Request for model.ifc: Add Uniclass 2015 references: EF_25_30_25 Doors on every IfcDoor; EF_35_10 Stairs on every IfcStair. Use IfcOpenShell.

First a look at what the model holds.

```python
import ifcopenshell

model = ifcopenshell.open("model.ifc")
print(model.schema)
print("classifications:", [c.Name for c in model.by_type("IfcClassification")])
for ifc_class in ("IfcDoor", "IfcRoof", "IfcStair", "IfcWall", "IfcWindow"):
    print(ifc_class, len(model.by_type(ifc_class)))
```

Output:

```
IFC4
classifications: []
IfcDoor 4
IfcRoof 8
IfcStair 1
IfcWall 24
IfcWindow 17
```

```python
import ifcopenshell
import ifcopenshell.api.classification

model = ifcopenshell.open("model.ifc")

system = ifcopenshell.api.classification.add_classification(model, classification="Uniclass 2015")

codes = {
    "IfcDoor": ("EF_25_30_25", "Doors"),
    "IfcStair": ("EF_35_10", "Stairs"),
}
for ifc_class, (code, name) in codes.items():
    products = model.by_type(ifc_class)
    ifcopenshell.api.classification.add_reference(
        model, products=products, classification=system, identification=code, name=name
    )
    print(code, len(products))

model.write("model-out.ifc")
```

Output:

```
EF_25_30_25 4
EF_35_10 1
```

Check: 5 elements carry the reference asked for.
